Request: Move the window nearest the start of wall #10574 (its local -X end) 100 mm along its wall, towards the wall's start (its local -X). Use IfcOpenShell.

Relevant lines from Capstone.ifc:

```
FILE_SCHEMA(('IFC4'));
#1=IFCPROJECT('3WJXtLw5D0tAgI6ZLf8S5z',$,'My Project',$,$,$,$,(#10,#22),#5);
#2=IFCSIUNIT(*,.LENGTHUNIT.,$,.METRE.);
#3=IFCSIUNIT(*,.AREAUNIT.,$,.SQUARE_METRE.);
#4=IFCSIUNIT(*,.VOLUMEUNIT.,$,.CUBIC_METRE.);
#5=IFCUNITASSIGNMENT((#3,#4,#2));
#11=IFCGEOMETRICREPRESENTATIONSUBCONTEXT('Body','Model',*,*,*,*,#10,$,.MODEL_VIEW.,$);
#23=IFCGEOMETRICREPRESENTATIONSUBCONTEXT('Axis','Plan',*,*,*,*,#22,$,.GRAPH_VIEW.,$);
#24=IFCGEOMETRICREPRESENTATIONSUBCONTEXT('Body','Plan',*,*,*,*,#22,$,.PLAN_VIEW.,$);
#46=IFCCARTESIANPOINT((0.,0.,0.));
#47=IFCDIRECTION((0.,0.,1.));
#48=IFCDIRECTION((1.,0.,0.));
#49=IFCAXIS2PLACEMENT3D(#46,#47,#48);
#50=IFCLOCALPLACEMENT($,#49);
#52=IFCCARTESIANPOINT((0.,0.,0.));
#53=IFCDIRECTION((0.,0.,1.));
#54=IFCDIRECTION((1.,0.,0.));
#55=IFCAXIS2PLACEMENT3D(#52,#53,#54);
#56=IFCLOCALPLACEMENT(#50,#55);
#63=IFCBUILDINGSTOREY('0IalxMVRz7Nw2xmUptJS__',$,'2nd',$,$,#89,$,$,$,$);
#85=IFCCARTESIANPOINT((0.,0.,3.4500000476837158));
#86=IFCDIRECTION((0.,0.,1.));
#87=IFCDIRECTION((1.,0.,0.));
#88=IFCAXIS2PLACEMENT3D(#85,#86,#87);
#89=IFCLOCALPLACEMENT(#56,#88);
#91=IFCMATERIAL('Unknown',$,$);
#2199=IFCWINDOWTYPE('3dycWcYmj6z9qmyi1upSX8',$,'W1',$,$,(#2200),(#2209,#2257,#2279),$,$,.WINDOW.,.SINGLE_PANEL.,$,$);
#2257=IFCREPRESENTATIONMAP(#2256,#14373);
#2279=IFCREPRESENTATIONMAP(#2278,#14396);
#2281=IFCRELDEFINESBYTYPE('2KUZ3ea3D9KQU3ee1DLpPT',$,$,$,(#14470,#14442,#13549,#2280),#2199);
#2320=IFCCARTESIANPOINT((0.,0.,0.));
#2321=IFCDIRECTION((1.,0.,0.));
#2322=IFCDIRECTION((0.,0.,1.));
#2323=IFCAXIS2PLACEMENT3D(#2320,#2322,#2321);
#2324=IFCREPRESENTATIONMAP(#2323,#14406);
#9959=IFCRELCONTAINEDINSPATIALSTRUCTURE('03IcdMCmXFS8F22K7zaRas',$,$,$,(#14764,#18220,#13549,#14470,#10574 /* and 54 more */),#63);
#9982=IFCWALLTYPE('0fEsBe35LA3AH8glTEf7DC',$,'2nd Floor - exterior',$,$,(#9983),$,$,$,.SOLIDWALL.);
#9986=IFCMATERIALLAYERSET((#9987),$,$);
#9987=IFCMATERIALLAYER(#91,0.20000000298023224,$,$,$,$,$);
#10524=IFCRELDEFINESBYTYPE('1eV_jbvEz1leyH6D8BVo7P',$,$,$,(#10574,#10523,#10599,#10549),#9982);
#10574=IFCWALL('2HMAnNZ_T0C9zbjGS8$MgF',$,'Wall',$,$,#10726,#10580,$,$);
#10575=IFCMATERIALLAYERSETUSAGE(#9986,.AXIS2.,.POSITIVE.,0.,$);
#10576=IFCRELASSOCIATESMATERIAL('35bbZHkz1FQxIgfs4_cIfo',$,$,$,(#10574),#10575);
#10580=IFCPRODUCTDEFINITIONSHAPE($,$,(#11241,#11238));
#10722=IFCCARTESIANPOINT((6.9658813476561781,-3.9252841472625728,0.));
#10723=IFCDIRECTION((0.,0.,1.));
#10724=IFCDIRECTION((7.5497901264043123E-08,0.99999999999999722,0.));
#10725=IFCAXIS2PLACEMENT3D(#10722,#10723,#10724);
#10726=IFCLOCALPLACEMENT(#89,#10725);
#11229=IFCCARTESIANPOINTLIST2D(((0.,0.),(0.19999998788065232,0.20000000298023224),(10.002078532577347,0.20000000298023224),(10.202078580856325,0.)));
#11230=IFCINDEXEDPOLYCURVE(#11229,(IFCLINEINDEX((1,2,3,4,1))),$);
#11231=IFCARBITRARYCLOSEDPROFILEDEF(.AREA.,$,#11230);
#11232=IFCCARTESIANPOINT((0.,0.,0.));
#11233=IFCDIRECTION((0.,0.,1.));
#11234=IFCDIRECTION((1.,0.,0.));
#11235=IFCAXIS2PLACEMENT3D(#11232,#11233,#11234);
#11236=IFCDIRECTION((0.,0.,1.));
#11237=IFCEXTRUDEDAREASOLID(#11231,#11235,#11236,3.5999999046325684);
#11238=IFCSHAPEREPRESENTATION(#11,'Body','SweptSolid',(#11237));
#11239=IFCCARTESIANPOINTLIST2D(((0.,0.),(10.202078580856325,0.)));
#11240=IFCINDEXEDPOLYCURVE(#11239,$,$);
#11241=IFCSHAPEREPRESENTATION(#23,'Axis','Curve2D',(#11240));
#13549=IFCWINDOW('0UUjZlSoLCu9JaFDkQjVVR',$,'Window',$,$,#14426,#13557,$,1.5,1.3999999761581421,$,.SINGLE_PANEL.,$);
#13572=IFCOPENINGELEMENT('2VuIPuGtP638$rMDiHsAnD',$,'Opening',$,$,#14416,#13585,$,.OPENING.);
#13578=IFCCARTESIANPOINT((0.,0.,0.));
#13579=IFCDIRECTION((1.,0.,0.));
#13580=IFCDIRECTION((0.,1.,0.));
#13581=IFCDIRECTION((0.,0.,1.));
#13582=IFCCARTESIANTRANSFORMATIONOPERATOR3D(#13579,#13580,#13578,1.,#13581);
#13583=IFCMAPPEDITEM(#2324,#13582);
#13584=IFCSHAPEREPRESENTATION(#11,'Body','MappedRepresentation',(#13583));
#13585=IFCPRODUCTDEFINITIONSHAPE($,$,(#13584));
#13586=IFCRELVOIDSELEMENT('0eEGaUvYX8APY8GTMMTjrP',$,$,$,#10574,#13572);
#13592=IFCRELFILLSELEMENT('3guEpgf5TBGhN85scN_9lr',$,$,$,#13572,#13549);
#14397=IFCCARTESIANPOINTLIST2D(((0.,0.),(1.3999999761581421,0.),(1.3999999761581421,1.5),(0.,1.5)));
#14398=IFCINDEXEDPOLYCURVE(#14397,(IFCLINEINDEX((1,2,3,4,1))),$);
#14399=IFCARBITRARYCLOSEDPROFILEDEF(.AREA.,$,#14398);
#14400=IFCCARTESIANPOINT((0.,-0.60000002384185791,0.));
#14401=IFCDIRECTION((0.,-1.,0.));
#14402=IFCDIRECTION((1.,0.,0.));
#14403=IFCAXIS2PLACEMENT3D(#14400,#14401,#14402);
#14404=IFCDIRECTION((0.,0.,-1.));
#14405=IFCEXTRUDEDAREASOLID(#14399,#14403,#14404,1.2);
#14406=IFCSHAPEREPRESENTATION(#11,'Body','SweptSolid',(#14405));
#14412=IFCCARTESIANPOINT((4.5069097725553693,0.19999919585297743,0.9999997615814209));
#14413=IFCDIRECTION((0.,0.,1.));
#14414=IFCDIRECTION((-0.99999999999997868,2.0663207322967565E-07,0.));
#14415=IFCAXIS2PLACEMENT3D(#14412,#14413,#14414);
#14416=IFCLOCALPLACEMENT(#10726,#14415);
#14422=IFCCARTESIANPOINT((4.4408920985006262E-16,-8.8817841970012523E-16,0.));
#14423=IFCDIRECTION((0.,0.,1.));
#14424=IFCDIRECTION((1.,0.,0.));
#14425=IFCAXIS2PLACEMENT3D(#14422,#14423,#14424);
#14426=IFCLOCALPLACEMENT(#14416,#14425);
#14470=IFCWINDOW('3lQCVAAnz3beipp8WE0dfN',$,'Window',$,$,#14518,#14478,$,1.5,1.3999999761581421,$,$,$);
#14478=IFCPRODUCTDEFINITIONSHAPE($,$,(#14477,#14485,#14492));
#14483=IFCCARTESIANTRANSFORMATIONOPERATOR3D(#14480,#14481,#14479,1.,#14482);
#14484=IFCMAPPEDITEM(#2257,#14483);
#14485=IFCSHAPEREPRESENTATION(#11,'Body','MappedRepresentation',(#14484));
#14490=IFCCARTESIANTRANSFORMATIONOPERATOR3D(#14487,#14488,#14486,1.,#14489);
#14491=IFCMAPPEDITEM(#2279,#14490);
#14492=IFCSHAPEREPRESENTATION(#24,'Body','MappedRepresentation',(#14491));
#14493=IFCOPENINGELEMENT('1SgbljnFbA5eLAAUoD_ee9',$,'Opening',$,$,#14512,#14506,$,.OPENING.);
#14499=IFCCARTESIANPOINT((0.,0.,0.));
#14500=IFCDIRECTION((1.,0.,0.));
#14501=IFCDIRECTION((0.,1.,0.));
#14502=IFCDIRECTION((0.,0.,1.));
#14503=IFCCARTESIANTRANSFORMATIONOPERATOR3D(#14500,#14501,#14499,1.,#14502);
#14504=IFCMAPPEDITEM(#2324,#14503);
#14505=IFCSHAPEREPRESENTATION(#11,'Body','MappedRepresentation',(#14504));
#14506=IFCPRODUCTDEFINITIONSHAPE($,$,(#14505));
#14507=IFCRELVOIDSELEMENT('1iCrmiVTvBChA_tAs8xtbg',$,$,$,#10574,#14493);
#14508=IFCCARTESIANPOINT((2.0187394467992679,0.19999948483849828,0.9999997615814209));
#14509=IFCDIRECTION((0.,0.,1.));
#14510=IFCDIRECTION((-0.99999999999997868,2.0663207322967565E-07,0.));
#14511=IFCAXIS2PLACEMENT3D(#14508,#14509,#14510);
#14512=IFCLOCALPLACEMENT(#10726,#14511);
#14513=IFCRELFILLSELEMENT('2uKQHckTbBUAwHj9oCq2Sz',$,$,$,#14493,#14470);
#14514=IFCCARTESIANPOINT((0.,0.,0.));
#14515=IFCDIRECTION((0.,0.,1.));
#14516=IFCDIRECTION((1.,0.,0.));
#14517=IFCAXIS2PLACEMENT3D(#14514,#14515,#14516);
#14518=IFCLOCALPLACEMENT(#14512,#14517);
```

```python
import ifcopenshell
import ifcopenshell.api.geometry
import ifcopenshell.util.placement

model = ifcopenshell.open("Capstone.ifc")

window = model.by_guid("3lQCVAAnz3beipp8WE0dfN")
opening = window.FillsVoids[0].RelatingOpeningElement
wall = opening.VoidsElements[0].RelatingBuildingElement

wall_matrix = ifcopenshell.util.placement.get_local_placement(wall.ObjectPlacement)
shift = wall_matrix[:3, 0] * -0.1
before = ifcopenshell.util.placement.get_local_placement(window.ObjectPlacement)[:3, 3].copy()

# The window is placed relative to its opening, so it follows when the opening moves.
matrix = ifcopenshell.util.placement.get_local_placement(opening.ObjectPlacement)
matrix[:3, 3] += shift
ifcopenshell.api.geometry.edit_object_placement(
    model, product=opening, matrix=matrix, is_si=False, should_transform_children=True
)

after = ifcopenshell.util.placement.get_local_placement(window.ObjectPlacement)[:3, 3]
print("window moved by", (after - before).round(3) + 0.0)

model.write("Capstone_edited.ifc")
```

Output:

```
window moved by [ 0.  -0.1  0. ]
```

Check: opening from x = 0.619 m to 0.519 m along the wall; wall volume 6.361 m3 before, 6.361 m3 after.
